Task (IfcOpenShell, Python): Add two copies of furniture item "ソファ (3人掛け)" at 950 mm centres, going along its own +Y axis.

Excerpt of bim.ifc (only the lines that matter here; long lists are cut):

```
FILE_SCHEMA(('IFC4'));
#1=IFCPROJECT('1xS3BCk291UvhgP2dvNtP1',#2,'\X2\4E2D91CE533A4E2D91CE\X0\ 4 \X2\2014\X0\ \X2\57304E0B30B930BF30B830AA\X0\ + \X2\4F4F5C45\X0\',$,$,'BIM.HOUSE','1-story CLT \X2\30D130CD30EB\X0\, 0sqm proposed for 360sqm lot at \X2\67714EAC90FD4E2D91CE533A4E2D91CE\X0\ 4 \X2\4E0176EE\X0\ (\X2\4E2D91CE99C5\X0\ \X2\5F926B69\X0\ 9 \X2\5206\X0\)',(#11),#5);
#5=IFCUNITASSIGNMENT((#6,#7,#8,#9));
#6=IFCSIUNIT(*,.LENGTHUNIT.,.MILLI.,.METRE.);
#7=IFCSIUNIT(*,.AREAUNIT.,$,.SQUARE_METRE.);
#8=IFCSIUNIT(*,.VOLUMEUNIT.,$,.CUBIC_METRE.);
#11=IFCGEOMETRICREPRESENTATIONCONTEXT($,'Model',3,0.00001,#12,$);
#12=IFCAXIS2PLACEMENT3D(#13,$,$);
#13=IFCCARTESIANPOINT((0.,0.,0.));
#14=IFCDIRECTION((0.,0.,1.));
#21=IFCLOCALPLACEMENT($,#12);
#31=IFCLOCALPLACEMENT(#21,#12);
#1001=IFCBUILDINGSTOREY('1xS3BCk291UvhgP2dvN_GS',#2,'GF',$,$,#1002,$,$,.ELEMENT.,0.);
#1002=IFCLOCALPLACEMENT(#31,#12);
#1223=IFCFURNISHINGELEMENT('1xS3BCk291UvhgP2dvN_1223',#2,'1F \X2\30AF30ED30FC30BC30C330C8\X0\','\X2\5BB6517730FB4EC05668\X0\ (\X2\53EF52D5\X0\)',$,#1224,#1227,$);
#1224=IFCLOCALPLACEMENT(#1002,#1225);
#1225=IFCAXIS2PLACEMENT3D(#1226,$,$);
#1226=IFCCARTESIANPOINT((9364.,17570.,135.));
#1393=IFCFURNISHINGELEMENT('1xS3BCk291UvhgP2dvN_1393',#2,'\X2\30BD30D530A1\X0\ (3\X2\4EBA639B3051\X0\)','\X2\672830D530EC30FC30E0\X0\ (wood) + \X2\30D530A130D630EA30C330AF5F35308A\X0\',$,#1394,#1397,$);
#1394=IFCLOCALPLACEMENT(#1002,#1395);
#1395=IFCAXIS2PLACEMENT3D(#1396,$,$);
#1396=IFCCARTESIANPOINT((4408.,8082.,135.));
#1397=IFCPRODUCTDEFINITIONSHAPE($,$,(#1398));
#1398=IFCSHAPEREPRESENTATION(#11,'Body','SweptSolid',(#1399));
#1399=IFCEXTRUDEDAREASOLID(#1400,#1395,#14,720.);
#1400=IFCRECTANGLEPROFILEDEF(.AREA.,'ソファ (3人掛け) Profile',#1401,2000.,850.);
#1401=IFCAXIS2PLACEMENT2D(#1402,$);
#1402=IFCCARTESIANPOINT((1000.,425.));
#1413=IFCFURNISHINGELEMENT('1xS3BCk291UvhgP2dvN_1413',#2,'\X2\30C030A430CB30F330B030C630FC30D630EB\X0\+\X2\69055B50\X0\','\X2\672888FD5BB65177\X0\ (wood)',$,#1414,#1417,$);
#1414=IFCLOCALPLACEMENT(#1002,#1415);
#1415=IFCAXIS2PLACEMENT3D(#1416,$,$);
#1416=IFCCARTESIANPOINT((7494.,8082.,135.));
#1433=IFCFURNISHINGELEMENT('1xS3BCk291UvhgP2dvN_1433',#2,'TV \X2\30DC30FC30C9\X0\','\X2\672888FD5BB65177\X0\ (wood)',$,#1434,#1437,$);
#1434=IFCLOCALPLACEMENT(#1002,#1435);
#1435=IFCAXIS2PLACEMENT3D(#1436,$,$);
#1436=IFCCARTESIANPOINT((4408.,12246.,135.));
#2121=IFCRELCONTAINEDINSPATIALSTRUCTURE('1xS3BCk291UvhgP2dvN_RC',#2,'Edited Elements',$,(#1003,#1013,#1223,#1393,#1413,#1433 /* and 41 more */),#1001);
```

```python
import ifcopenshell
import ifcopenshell.api.geometry
import ifcopenshell.api.root
import ifcopenshell.util.element
import ifcopenshell.util.placement
import ifcopenshell.util.unit

model = ifcopenshell.open("bim.ifc")
unit_scale = ifcopenshell.util.unit.calculate_unit_scale(model)


def reuse_history(source, copy):
    """copy_class also copies each property set's owner history, people and application; keep the originals."""
    for rel in copy.IsDefinedBy:
        if rel.is_a("IfcRelDefinesByProperties") and (history := rel.RelatingPropertyDefinition.OwnerHistory):
            rel.RelatingPropertyDefinition.OwnerHistory = source.OwnerHistory
            ifcopenshell.util.element.remove_deep2(model, history)


source = model.by_id(1393)
base = ifcopenshell.util.placement.get_local_placement(source.ObjectPlacement)
step = base[:3, 1] * 0.95 / unit_scale

for i in range(1, 3):
    copy = ifcopenshell.api.root.copy_class(model, product=source)
    copy.Representation = ifcopenshell.util.element.copy_deep(
        model, source.Representation, exclude=["IfcGeometricRepresentationContext", "IfcRepresentationMap"]
    )
    reuse_history(source, copy)
    matrix = base.copy()
    matrix[:3, 3] += i * step
    print("added at", matrix[:3, 3].round(3) + 0.0)
    ifcopenshell.api.geometry.edit_object_placement(model, product=copy, matrix=matrix, is_si=False)

model.write("bim_edited.ifc")
```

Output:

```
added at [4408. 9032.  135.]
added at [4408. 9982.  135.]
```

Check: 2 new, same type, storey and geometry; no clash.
